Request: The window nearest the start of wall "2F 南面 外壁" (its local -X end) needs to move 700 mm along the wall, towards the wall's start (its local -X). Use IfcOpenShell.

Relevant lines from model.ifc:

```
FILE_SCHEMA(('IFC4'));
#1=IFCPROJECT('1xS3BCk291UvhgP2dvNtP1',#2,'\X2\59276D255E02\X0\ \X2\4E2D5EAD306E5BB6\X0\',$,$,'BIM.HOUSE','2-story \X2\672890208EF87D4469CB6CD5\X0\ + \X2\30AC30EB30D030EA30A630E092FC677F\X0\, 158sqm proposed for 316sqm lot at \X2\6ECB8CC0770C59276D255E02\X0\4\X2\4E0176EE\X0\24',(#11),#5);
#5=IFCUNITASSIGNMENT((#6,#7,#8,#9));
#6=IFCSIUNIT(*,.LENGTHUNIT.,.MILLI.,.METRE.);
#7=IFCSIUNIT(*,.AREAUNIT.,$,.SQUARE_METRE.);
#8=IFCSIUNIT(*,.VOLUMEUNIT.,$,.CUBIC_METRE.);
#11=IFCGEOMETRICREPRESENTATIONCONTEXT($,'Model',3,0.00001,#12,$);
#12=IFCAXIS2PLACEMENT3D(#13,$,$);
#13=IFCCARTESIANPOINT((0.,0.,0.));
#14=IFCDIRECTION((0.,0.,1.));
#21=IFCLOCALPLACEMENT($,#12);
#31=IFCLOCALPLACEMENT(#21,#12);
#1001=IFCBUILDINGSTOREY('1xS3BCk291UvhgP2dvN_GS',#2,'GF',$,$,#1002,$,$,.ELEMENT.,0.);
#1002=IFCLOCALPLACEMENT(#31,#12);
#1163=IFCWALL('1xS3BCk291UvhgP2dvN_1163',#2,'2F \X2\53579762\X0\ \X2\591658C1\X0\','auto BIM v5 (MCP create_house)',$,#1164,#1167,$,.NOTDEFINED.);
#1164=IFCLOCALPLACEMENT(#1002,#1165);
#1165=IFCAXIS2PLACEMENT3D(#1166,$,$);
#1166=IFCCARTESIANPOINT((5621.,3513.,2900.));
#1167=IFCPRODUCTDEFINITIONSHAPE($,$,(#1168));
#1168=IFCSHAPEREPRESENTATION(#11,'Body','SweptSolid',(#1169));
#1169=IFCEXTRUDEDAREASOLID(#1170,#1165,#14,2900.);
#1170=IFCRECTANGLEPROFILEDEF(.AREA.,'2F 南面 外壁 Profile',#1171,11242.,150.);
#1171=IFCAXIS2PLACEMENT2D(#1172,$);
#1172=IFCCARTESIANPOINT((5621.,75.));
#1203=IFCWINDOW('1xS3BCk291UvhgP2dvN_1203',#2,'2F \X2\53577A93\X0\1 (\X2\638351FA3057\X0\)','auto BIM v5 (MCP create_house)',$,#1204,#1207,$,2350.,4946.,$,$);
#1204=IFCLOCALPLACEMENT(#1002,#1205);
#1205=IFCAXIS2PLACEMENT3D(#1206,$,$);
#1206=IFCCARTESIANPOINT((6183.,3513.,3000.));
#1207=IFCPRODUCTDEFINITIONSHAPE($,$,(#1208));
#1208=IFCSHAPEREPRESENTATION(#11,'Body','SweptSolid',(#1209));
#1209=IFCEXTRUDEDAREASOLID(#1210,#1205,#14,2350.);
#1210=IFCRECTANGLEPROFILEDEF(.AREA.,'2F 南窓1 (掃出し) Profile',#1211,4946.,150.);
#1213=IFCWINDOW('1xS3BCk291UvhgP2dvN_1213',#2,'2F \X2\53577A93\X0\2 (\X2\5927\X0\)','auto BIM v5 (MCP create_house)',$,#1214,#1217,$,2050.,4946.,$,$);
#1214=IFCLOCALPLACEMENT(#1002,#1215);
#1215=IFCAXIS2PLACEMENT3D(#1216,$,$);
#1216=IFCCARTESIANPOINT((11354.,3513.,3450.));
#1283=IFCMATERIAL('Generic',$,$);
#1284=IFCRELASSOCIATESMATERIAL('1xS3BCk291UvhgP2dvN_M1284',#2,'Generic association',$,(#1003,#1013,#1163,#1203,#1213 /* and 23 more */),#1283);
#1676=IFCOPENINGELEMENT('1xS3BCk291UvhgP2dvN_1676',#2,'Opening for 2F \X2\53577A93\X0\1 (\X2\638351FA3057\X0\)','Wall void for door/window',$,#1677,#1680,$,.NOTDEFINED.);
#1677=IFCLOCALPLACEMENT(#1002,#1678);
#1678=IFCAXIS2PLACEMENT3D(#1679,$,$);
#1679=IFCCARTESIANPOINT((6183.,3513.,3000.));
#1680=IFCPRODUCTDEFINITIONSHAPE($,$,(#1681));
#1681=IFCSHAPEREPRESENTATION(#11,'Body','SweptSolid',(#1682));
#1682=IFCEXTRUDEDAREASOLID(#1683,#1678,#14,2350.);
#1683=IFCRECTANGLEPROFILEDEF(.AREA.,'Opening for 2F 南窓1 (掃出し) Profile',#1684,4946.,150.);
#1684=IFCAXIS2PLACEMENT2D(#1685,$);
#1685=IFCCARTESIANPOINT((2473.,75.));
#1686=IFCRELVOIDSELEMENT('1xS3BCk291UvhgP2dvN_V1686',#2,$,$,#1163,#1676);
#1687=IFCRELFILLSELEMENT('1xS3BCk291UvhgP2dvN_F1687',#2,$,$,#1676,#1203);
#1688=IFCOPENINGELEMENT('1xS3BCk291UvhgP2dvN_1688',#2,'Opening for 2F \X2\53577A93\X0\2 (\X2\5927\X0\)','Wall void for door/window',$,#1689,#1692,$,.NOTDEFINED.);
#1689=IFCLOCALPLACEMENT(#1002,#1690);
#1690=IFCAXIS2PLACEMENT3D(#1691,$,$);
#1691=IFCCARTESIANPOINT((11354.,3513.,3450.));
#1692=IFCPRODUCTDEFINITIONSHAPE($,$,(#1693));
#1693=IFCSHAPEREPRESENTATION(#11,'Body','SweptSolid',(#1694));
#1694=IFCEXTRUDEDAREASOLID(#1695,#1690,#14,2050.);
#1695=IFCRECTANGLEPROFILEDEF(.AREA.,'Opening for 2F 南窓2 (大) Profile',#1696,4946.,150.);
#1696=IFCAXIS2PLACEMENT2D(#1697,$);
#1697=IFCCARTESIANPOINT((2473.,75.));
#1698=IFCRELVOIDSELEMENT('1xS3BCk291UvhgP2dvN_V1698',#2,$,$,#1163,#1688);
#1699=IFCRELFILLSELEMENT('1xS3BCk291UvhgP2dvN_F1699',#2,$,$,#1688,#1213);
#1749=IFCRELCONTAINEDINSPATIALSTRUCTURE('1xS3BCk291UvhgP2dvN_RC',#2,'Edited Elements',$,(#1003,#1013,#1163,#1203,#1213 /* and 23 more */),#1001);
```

```python
import ifcopenshell
import ifcopenshell.api.geometry
import ifcopenshell.util.placement

model = ifcopenshell.open("model.ifc")

window = model.by_guid("1xS3BCk291UvhgP2dvN_1203")
opening = window.FillsVoids[0].RelatingOpeningElement
wall = opening.VoidsElements[0].RelatingBuildingElement

wall_matrix = ifcopenshell.util.placement.get_local_placement(wall.ObjectPlacement)
shift = wall_matrix[:3, 0] * -700.0
before = ifcopenshell.util.placement.get_local_placement(window.ObjectPlacement)[:3, 3].copy()

# The window is not placed relative to its opening, so move both.
for product in (opening, window):
    matrix = ifcopenshell.util.placement.get_local_placement(product.ObjectPlacement)
    matrix[:3, 3] += shift
    ifcopenshell.api.geometry.edit_object_placement(model, product=product, matrix=matrix, is_si=False)

after = ifcopenshell.util.placement.get_local_placement(window.ObjectPlacement)[:3, 3]
print("window moved by", (after - before).round(3) + 0.0)

model.write("model-out.ifc")
```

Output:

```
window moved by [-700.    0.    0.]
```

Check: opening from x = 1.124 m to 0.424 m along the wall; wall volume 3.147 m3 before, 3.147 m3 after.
